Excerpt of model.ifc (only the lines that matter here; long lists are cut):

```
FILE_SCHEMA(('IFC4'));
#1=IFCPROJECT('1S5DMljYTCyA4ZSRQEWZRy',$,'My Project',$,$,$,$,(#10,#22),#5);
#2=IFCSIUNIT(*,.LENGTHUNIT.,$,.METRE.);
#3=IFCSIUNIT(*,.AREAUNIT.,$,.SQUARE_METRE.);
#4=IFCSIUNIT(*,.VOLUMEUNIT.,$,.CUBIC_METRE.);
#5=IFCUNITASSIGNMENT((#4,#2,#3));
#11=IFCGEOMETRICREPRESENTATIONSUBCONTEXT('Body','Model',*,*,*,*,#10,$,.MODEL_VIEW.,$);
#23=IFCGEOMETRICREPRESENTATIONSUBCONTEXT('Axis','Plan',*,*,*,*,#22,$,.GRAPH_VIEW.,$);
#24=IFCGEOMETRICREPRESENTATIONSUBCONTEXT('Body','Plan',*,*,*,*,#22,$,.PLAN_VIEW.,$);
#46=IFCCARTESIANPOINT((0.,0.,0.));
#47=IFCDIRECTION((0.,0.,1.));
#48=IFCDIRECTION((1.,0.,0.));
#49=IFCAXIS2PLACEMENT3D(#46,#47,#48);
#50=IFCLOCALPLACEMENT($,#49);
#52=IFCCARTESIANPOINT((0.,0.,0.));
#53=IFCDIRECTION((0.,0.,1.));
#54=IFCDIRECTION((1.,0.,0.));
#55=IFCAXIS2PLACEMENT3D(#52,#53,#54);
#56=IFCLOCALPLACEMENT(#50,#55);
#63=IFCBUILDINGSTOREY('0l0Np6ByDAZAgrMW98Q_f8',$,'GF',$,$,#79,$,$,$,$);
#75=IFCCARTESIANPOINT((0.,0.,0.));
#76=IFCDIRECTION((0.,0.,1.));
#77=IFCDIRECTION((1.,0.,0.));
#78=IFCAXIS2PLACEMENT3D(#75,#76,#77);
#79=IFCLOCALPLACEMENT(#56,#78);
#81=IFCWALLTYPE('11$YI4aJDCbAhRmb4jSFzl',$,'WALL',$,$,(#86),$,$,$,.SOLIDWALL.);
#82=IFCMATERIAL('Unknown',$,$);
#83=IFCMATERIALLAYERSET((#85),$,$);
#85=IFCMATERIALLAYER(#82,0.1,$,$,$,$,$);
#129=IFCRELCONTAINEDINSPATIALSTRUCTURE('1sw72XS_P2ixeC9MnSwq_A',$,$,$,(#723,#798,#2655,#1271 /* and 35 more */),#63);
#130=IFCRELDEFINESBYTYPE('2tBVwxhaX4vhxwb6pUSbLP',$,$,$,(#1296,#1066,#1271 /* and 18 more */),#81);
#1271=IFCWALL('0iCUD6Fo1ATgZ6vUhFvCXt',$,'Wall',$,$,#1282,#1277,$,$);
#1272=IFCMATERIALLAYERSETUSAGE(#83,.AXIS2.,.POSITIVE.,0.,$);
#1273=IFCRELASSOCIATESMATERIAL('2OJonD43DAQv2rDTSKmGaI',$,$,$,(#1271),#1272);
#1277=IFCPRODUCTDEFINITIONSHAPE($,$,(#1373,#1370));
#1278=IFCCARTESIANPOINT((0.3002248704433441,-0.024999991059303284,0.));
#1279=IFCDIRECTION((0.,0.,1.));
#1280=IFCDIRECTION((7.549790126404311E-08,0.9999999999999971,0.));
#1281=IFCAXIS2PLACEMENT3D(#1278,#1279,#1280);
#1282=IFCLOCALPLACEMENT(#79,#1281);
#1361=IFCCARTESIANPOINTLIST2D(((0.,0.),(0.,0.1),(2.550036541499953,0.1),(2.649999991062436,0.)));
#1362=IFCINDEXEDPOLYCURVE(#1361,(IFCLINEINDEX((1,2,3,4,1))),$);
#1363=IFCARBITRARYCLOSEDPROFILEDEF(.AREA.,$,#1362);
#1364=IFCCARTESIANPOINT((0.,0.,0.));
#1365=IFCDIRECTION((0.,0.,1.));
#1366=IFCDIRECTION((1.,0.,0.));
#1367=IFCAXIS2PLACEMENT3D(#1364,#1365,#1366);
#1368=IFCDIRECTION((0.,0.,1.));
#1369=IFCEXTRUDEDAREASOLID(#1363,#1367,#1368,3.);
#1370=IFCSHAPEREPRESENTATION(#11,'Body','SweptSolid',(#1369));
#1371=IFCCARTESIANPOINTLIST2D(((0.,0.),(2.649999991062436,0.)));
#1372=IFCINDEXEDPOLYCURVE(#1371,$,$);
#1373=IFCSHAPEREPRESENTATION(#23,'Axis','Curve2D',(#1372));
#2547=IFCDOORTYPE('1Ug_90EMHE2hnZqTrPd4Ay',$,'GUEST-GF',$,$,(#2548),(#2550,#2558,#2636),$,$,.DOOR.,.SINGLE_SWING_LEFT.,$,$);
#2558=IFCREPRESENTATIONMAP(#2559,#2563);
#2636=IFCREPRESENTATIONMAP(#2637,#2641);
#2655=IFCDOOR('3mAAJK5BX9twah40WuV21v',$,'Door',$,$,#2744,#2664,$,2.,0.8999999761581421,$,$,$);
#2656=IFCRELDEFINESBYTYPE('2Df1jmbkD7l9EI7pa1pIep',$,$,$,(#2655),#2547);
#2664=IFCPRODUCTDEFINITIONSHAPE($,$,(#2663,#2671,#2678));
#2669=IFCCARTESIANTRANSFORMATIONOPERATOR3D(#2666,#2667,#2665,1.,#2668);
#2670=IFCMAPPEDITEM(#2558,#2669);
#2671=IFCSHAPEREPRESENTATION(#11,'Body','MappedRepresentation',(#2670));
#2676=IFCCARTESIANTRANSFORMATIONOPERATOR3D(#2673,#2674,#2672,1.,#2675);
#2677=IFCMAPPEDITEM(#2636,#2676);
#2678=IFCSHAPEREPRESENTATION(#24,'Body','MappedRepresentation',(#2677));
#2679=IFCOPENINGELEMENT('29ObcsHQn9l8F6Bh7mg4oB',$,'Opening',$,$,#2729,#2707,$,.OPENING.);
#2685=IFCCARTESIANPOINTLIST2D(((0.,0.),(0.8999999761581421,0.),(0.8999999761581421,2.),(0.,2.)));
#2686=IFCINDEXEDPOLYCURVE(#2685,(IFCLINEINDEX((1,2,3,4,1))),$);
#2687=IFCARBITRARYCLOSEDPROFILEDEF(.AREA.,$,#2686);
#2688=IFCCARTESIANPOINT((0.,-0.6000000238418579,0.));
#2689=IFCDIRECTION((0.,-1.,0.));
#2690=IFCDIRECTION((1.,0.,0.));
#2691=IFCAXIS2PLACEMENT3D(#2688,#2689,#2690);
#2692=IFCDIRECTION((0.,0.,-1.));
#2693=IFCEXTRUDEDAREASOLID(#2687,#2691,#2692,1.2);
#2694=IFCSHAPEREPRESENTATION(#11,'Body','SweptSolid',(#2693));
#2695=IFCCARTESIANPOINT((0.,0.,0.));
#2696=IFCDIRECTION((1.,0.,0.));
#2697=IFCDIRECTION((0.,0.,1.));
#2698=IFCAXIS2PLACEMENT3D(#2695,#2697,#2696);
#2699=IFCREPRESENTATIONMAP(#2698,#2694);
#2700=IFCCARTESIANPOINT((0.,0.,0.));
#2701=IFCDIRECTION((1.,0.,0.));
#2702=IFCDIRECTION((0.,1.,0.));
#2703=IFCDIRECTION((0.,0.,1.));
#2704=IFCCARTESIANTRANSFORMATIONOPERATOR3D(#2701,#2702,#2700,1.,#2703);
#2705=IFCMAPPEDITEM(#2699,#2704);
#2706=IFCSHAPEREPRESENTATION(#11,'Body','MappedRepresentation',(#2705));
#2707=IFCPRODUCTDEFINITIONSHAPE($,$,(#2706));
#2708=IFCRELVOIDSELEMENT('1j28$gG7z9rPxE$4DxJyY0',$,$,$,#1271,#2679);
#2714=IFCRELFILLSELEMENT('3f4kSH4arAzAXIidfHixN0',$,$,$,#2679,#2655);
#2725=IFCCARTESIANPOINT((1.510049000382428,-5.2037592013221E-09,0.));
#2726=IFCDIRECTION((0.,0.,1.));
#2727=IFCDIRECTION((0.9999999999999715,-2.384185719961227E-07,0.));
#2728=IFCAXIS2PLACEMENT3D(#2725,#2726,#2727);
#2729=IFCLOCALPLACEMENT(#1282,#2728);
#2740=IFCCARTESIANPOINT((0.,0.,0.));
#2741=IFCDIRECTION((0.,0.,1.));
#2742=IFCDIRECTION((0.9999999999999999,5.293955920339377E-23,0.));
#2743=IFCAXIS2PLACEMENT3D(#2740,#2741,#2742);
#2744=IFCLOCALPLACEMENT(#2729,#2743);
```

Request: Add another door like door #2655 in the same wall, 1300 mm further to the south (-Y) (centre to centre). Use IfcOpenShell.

```python
import ifcopenshell
import ifcopenshell.api.feature
import ifcopenshell.api.geometry
import ifcopenshell.api.root
import ifcopenshell.geom
import ifcopenshell.util.element
import ifcopenshell.util.placement
import ifcopenshell.util.shape

model = ifcopenshell.open("model.ifc")
settings = ifcopenshell.geom.settings()


def volume(element):
    """Net volume in cubic metres, openings subtracted."""
    shape = ifcopenshell.geom.create_shape(settings, element)
    return ifcopenshell.util.shape.get_volume(shape.geometry)


door = model.by_guid("3mAAJK5BX9twah40WuV21v")
opening = door.FillsVoids[0].RelatingOpeningElement
wall = opening.VoidsElements[0].RelatingBuildingElement
before = volume(wall)
shift = ifcopenshell.util.placement.get_local_placement(wall.ObjectPlacement)[:3, 0] * -1.3

# copy_class copies the void relationship, type, container and properties, but no geometry.
new_opening = ifcopenshell.api.root.copy_class(model, product=opening)
new_opening.Representation = ifcopenshell.util.element.copy_deep(
    model, opening.Representation, exclude=["IfcGeometricRepresentationContext", "IfcRepresentationMap"]
)
new_door = ifcopenshell.api.root.copy_class(model, product=door)
new_door.Representation = ifcopenshell.util.element.copy_deep(
    model, door.Representation, exclude=["IfcGeometricRepresentationContext", "IfcRepresentationMap"]
)
ifcopenshell.api.feature.add_filling(model, opening=new_opening, element=new_door)

for old, new in ((opening, new_opening), (door, new_door)):
    matrix = ifcopenshell.util.placement.get_local_placement(old.ObjectPlacement)
    matrix[:3, 3] += shift
    ifcopenshell.api.geometry.edit_object_placement(model, product=new, matrix=matrix, is_si=False)

after = volume(wall)

print(f"wall volume {before:.3f} -> {after:.3f} m3")

model.write("model-out.ifc")
```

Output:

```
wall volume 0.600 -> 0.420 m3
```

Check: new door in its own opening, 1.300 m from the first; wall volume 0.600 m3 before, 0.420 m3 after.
